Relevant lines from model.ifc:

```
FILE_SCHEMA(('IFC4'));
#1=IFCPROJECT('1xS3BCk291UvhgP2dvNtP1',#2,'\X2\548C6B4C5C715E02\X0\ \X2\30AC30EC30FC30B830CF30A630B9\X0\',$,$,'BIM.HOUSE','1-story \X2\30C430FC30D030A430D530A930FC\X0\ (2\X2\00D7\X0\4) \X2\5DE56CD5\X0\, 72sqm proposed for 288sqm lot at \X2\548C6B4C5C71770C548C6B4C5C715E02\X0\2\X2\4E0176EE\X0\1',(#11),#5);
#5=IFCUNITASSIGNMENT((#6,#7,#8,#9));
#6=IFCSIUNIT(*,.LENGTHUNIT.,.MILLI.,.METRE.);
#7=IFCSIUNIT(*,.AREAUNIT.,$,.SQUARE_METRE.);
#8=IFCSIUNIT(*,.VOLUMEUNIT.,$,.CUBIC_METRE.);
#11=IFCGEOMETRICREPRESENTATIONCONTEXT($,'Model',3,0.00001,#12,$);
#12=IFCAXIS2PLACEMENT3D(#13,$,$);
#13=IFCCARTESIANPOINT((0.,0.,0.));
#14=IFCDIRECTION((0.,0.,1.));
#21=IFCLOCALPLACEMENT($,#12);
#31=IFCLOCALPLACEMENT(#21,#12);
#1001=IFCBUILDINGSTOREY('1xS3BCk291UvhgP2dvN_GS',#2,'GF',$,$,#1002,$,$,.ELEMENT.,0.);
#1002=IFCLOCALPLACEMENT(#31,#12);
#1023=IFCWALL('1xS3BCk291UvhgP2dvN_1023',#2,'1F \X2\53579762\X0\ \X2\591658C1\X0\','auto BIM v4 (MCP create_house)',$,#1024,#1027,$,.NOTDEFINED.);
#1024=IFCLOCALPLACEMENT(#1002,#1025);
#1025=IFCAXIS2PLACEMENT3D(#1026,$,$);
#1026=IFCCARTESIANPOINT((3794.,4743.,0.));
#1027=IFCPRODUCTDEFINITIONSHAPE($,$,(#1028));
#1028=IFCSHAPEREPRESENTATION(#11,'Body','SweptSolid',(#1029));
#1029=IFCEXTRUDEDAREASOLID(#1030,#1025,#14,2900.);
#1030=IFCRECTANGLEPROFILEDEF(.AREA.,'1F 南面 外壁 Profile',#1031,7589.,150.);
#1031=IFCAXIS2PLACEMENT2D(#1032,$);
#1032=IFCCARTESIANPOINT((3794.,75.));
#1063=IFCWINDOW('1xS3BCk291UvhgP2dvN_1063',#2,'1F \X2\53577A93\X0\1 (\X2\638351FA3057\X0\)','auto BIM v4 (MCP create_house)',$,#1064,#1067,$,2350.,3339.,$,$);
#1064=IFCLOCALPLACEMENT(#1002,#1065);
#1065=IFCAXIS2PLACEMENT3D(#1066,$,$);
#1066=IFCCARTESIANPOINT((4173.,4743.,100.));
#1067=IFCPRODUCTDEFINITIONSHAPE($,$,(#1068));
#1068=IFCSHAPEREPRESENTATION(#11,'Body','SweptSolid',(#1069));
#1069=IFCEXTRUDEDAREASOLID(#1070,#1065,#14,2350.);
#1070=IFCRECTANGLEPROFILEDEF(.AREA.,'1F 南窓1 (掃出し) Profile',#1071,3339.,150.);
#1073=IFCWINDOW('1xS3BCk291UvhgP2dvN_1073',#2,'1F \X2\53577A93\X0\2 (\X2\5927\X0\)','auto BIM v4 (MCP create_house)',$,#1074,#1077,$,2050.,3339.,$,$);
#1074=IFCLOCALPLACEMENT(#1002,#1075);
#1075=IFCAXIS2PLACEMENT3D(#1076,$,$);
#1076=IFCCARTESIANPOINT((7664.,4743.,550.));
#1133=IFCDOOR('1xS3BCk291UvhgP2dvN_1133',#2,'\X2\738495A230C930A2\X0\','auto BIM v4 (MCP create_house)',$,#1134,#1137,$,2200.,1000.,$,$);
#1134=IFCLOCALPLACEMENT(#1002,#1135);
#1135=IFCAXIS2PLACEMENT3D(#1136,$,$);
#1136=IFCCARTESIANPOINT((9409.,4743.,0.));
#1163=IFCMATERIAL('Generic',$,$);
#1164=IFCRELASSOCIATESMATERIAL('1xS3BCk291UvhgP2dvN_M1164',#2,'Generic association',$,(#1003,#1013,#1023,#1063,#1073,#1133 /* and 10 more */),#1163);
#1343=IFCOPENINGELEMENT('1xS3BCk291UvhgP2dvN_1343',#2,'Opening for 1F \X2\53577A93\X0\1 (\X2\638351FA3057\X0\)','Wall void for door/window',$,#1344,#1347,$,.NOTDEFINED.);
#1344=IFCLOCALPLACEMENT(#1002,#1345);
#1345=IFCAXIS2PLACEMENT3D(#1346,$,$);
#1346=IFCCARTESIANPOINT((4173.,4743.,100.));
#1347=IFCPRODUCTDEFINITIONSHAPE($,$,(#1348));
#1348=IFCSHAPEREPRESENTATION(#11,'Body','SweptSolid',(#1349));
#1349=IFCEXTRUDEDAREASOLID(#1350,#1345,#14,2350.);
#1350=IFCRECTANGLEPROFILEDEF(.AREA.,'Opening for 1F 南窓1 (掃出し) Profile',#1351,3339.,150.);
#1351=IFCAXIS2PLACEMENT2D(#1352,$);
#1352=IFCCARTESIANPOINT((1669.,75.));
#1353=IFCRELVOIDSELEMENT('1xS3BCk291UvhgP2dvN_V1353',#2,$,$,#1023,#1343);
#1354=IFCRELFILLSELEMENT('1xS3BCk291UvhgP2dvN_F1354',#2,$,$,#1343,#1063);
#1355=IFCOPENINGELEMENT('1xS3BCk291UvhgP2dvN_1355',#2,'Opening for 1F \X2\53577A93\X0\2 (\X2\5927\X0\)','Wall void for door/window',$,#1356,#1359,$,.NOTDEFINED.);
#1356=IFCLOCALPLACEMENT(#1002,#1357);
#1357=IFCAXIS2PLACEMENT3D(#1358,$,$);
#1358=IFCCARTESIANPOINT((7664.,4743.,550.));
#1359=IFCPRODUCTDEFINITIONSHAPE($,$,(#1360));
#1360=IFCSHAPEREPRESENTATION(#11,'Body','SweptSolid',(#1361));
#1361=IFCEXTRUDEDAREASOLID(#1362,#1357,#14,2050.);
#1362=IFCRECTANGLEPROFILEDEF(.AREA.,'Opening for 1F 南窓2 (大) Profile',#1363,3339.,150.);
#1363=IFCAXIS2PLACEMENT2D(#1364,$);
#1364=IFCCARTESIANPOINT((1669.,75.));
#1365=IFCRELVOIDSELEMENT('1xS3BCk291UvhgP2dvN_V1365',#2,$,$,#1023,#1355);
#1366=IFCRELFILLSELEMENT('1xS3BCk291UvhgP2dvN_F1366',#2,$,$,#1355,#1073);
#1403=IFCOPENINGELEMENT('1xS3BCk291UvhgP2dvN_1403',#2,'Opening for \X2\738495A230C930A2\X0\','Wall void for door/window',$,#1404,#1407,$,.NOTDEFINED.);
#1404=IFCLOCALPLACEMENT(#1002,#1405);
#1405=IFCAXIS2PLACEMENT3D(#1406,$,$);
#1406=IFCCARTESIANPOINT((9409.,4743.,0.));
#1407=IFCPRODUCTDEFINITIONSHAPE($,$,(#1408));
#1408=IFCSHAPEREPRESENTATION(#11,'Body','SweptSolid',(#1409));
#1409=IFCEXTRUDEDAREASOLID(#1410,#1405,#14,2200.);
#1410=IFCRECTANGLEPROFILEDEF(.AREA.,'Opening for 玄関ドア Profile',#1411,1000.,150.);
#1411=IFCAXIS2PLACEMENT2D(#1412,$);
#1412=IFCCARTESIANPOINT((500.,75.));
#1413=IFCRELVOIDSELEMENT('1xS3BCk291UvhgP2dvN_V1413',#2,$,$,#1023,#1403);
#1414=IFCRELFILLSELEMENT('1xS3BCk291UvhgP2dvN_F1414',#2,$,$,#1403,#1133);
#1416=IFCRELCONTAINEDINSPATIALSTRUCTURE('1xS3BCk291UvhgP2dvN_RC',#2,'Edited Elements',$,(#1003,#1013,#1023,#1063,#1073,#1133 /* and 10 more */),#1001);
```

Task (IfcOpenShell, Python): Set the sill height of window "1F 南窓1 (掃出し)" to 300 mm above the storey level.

```python
import numpy as np
import ifcopenshell
import ifcopenshell.api.geometry
import ifcopenshell.geom
import ifcopenshell.util.element
import ifcopenshell.util.placement
import ifcopenshell.util.shape
import ifcopenshell.util.unit

model = ifcopenshell.open("model.ifc")
unit_scale = ifcopenshell.util.unit.calculate_unit_scale(model)

window = model.by_guid("1xS3BCk291UvhgP2dvN_1063")
opening = window.FillsVoids[0].RelatingOpeningElement
storey = ifcopenshell.util.element.get_container(window, ifc_class="IfcBuildingStorey")
level = ifcopenshell.util.placement.get_local_placement(storey.ObjectPlacement)[2, 3]

# The opening's origin need not be at the sill, so measure its lowest point.
shape = ifcopenshell.geom.create_shape(ifcopenshell.geom.settings(), opening)
bottom = ifcopenshell.util.shape.get_shape_bottom_elevation(shape, shape.geometry) / unit_scale
dz = level + 300.0 - bottom

shift = np.array([0.0, 0.0, dz])
# The window is not placed relative to its opening, so move both.
for product in (opening, window):
    matrix = ifcopenshell.util.placement.get_local_placement(product.ObjectPlacement)
    matrix[:3, 3] += shift
    ifcopenshell.api.geometry.edit_object_placement(model, product=product, matrix=matrix, is_si=False)

print(f"moved by {dz * unit_scale:+.3f} m")

model.write("model-out.ifc")
```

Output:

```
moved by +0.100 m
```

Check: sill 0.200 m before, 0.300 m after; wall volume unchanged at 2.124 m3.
